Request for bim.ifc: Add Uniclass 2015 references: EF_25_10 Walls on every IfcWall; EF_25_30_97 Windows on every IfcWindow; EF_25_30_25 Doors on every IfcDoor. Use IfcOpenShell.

First a look at what the model holds.

```python
import ifcopenshell

model = ifcopenshell.open("bim.ifc")
print(model.schema)
print("classifications:", [c.Name for c in model.by_type("IfcClassification")])
for ifc_class in ("IfcDoor", "IfcRoof", "IfcStair", "IfcWall", "IfcWindow"):
    print(ifc_class, len(model.by_type(ifc_class)))
```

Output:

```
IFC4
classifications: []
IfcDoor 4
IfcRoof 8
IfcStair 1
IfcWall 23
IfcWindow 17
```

```python
import ifcopenshell
import ifcopenshell.api.classification

model = ifcopenshell.open("bim.ifc")

system = ifcopenshell.api.classification.add_classification(model, classification="Uniclass 2015")

codes = {
    "IfcWall": ("EF_25_10", "Walls"),
    "IfcWindow": ("EF_25_30_97", "Windows"),
    "IfcDoor": ("EF_25_30_25", "Doors"),
}
for ifc_class, (code, name) in codes.items():
    products = model.by_type(ifc_class)
    ifcopenshell.api.classification.add_reference(
        model, products=products, classification=system, identification=code, name=name
    )
    print(code, len(products))

model.write("bim_updated.ifc")
```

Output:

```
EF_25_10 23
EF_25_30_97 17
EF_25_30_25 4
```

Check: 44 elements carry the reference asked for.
